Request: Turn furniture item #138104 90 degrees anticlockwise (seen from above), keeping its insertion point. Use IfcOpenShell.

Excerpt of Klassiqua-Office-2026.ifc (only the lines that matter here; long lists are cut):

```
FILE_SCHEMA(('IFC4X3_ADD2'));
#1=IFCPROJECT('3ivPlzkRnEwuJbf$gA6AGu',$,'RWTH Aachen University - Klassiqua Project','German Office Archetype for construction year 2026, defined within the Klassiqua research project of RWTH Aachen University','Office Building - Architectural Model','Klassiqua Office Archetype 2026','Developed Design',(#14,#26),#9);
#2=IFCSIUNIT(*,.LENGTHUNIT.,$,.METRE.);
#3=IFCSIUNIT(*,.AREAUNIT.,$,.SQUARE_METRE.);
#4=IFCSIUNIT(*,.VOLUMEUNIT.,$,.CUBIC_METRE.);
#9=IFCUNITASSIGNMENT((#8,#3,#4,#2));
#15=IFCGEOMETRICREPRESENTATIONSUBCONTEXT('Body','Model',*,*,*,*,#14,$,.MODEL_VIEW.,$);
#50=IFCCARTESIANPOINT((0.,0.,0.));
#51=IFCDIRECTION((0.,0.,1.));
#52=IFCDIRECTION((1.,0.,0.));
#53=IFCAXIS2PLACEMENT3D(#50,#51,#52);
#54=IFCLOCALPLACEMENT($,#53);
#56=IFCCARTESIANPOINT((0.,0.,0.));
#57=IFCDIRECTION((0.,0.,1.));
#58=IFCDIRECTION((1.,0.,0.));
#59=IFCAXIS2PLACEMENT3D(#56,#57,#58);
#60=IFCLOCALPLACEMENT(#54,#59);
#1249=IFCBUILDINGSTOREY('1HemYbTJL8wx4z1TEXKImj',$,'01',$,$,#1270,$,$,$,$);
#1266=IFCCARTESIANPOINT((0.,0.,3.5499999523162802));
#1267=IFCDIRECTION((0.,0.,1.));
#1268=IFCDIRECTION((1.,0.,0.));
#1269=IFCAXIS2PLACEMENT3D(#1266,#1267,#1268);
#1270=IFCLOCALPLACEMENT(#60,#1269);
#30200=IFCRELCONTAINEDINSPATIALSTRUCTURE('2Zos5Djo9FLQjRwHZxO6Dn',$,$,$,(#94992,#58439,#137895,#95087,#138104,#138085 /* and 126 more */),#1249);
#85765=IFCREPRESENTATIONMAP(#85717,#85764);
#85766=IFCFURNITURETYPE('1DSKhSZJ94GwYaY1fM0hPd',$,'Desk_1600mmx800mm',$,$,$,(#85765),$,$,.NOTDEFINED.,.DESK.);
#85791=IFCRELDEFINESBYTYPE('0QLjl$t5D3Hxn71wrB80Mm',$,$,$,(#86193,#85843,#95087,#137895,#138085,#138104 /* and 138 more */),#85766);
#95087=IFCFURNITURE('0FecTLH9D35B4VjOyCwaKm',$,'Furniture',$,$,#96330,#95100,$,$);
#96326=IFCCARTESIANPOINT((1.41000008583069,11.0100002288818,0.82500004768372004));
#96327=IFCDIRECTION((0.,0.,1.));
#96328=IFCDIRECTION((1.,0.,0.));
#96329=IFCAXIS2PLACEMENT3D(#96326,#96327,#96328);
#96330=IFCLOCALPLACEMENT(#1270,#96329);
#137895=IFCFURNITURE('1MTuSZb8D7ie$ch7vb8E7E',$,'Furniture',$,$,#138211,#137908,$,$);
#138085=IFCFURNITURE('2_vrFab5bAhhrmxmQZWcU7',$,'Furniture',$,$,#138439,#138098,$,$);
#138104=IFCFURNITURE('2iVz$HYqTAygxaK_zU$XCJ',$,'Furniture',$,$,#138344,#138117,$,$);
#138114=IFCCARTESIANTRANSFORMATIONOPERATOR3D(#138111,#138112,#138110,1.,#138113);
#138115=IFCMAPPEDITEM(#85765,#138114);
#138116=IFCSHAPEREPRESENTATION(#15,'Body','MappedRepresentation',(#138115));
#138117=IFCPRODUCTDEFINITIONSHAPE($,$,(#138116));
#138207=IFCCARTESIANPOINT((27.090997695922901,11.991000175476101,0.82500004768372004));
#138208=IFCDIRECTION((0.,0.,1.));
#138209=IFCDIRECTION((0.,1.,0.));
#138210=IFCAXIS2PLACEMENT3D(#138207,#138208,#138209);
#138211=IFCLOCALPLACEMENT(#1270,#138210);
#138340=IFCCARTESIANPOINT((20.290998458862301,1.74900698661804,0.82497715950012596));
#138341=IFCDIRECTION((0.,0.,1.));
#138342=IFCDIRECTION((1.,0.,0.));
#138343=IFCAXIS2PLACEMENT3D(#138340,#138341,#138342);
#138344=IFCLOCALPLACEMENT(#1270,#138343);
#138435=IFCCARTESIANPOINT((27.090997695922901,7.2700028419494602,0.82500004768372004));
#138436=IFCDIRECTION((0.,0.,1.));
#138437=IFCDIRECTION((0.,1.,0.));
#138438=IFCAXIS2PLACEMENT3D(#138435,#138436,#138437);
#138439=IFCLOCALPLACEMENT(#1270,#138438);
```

```python
import ifcopenshell
import ifcopenshell.api.geometry
import ifcopenshell.util.placement

model = ifcopenshell.open("Klassiqua-Office-2026.ifc")

item = model.by_guid("2iVz$HYqTAygxaK_zU$XCJ")
matrix = ifcopenshell.util.placement.get_local_placement(item.ObjectPlacement)
matrix = matrix @ ifcopenshell.util.placement.rotation(90, "Z")
ifcopenshell.api.geometry.edit_object_placement(model, product=item, matrix=matrix, is_si=False)

print(ifcopenshell.util.placement.get_local_placement(item.ObjectPlacement).round(3) + 0.0)

model.write("Klassiqua-Office-2026_updated.ifc")
```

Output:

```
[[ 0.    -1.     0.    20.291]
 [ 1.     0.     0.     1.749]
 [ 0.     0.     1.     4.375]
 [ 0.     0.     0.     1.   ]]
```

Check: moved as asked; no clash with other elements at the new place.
